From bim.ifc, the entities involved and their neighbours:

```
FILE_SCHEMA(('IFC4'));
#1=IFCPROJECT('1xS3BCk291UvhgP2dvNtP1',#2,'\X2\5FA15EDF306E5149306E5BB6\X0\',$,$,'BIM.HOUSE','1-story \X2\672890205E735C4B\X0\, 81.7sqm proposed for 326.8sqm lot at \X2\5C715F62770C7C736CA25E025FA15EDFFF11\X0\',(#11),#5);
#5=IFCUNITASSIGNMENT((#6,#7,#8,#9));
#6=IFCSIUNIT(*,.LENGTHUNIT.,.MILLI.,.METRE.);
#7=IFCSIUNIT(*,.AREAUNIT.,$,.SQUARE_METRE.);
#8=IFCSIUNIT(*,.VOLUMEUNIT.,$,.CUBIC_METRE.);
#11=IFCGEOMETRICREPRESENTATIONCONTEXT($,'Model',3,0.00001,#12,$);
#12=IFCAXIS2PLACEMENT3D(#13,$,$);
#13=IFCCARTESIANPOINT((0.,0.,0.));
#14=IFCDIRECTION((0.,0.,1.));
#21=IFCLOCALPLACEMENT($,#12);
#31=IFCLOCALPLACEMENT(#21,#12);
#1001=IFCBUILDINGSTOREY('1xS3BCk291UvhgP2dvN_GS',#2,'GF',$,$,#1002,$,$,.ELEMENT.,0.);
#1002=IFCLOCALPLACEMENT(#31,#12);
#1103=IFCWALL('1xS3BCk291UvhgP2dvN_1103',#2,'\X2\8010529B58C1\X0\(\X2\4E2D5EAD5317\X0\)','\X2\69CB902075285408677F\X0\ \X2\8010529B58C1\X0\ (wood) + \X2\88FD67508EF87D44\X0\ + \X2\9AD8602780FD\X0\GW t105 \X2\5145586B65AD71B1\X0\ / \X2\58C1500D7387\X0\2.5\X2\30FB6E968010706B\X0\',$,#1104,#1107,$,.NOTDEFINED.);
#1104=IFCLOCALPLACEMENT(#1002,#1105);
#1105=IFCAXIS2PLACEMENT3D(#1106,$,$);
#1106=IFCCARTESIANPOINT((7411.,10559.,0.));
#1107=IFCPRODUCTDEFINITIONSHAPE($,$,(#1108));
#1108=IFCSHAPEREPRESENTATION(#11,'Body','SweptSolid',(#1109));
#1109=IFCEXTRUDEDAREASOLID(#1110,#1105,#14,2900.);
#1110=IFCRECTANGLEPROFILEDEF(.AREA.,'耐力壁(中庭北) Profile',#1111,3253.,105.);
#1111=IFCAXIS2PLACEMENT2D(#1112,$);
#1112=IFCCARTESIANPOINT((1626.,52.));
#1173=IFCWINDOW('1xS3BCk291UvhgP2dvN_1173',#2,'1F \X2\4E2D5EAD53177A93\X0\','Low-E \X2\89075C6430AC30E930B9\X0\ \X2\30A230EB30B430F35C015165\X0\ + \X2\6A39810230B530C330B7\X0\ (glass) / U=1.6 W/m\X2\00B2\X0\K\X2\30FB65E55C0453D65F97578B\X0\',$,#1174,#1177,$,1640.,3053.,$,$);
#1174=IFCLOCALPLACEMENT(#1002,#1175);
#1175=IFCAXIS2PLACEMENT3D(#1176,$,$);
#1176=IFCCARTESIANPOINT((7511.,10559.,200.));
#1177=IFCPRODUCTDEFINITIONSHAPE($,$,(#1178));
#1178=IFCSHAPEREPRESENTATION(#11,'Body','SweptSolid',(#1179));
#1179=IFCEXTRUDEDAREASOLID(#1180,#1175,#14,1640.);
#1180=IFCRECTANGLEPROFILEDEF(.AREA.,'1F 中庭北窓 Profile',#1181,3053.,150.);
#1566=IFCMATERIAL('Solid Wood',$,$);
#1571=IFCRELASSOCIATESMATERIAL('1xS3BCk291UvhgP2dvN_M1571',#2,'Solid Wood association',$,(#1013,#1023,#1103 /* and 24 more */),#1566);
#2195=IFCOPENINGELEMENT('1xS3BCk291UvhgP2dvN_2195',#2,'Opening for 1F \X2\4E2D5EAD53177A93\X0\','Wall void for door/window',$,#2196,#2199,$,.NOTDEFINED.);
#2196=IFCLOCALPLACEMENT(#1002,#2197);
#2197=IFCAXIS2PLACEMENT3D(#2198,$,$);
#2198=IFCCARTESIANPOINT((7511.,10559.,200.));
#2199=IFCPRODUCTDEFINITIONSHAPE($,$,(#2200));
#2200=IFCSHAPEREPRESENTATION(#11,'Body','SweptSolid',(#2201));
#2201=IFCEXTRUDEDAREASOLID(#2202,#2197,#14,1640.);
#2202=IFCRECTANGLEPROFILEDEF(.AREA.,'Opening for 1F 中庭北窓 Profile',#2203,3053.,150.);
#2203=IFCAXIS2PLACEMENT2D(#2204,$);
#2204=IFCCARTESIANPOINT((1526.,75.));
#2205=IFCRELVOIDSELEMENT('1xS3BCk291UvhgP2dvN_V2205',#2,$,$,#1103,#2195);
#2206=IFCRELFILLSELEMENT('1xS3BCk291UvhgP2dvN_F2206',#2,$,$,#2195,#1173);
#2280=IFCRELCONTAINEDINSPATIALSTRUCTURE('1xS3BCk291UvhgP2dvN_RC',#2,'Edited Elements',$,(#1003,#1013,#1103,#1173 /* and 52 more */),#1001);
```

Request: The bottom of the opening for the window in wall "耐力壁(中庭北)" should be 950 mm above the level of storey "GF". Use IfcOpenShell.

```python
import numpy as np
import ifcopenshell
import ifcopenshell.api.geometry
import ifcopenshell.geom
import ifcopenshell.util.element
import ifcopenshell.util.placement
import ifcopenshell.util.shape
import ifcopenshell.util.unit

model = ifcopenshell.open("bim.ifc")
unit_scale = ifcopenshell.util.unit.calculate_unit_scale(model)

window = model.by_guid("1xS3BCk291UvhgP2dvN_1173")
opening = window.FillsVoids[0].RelatingOpeningElement
storey = ifcopenshell.util.element.get_container(window, ifc_class="IfcBuildingStorey")
level = ifcopenshell.util.placement.get_local_placement(storey.ObjectPlacement)[2, 3]

# The opening's origin need not be at the sill, so measure its lowest point.
shape = ifcopenshell.geom.create_shape(ifcopenshell.geom.settings(), opening)
bottom = ifcopenshell.util.shape.get_shape_bottom_elevation(shape, shape.geometry) / unit_scale
dz = level + 0.95 / unit_scale - bottom

shift = np.array([0.0, 0.0, dz])
# The window is not placed relative to its opening, so move both.
for product in (opening, window):
    matrix = ifcopenshell.util.placement.get_local_placement(product.ObjectPlacement)
    matrix[:3, 3] += shift
    ifcopenshell.api.geometry.edit_object_placement(model, product=product, matrix=matrix, is_si=False)

print(f"moved by {dz * unit_scale:+.3f} m")

model.write("bim_v2.ifc")
```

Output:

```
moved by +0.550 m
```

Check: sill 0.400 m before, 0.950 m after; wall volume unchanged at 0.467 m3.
